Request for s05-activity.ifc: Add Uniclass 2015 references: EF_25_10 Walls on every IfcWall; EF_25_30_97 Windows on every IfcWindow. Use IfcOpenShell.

First a look at what the model holds.

```python
import ifcopenshell

model = ifcopenshell.open("s05-activity.ifc")
print(model.schema)
print("classifications:", [c.Name for c in model.by_type("IfcClassification")])
for ifc_class in ("IfcDoor", "IfcRoof", "IfcStair", "IfcWall", "IfcWindow"):
    print(ifc_class, len(model.by_type(ifc_class)))
```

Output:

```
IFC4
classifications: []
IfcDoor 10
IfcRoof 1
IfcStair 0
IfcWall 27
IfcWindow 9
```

```python
import ifcopenshell
import ifcopenshell.api.classification

model = ifcopenshell.open("s05-activity.ifc")

system = ifcopenshell.api.classification.add_classification(model, classification="Uniclass 2015")

codes = {
    "IfcWall": ("EF_25_10", "Walls"),
    "IfcWindow": ("EF_25_30_97", "Windows"),
}
for ifc_class, (code, name) in codes.items():
    products = model.by_type(ifc_class)
    ifcopenshell.api.classification.add_reference(
        model, products=products, classification=system, identification=code, name=name
    )
    print(code, len(products))

model.write("s05-activity-out.ifc")
```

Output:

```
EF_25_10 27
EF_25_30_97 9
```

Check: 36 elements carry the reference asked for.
